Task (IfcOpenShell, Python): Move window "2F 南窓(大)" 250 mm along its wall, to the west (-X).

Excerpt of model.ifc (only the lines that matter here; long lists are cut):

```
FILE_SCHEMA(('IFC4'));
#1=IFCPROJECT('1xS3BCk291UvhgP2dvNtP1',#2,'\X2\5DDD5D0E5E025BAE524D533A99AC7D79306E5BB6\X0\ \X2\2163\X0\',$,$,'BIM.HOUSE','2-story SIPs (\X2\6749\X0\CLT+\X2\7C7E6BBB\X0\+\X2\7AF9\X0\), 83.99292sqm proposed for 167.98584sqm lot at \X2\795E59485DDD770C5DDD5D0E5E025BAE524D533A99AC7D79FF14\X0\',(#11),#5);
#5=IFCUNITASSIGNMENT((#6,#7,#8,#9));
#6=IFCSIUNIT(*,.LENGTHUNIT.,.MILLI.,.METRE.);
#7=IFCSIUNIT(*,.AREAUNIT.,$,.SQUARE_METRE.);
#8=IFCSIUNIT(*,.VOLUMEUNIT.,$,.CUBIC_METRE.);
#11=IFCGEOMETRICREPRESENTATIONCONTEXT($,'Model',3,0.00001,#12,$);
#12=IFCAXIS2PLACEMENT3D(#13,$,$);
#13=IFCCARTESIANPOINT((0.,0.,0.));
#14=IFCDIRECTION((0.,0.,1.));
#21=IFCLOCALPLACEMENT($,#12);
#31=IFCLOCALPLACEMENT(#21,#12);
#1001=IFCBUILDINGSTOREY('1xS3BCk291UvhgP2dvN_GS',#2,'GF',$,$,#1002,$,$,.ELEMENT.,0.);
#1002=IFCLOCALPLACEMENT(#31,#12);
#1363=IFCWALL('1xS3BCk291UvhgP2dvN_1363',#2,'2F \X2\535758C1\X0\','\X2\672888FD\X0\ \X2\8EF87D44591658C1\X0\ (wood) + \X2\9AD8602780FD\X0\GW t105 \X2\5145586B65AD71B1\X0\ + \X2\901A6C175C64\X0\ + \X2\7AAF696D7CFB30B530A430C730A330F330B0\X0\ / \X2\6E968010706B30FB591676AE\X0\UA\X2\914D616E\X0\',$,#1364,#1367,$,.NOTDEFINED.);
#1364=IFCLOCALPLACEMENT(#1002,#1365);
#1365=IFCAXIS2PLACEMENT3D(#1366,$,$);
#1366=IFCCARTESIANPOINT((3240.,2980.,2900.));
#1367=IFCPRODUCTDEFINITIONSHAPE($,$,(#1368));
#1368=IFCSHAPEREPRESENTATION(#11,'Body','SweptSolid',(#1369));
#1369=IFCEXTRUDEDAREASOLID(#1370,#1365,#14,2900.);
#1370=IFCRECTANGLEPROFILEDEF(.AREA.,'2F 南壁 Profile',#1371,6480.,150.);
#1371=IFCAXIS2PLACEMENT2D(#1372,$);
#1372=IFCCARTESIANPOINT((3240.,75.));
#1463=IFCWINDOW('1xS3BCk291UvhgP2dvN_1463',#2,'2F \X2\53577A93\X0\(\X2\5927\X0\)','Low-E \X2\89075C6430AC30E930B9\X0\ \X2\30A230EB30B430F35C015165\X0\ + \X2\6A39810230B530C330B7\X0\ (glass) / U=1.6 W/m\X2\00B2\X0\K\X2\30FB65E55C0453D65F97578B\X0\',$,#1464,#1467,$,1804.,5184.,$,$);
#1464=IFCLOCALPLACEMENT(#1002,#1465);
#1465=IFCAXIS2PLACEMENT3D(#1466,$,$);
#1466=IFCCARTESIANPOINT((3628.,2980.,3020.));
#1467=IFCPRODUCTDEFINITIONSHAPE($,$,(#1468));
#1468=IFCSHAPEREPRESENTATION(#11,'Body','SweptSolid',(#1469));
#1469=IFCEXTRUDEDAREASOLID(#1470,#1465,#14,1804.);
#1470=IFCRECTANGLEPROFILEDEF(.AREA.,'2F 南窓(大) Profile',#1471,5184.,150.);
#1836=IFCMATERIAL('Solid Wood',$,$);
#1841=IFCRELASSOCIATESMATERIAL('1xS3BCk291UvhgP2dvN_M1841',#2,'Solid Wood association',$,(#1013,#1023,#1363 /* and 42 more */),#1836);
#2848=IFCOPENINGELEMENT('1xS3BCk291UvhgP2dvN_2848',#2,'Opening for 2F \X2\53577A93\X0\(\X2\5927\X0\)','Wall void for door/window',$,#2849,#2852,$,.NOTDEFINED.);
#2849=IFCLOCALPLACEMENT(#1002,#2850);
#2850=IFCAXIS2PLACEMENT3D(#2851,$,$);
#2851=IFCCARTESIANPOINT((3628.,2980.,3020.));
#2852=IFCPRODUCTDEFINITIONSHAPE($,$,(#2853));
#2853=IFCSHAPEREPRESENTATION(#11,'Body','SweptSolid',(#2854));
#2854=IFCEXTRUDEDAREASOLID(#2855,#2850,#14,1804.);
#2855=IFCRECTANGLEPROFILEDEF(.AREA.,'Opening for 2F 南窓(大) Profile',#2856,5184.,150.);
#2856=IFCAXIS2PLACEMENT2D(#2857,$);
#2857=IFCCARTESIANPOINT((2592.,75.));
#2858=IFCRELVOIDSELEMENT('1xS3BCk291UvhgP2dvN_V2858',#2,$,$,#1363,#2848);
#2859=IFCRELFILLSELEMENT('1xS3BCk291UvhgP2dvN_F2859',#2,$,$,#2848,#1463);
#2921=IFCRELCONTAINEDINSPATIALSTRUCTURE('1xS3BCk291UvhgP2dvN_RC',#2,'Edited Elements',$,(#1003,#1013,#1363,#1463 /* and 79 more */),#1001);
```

```python
import ifcopenshell
import ifcopenshell.api.geometry
import ifcopenshell.util.placement
import ifcopenshell.util.unit

model = ifcopenshell.open("model.ifc")
unit_scale = ifcopenshell.util.unit.calculate_unit_scale(model)

window = model.by_guid("1xS3BCk291UvhgP2dvN_1463")
opening = window.FillsVoids[0].RelatingOpeningElement
wall = opening.VoidsElements[0].RelatingBuildingElement

wall_matrix = ifcopenshell.util.placement.get_local_placement(wall.ObjectPlacement)
shift = wall_matrix[:3, 0] * -0.25 / unit_scale
before = ifcopenshell.util.placement.get_local_placement(window.ObjectPlacement)[:3, 3].copy()

# The window is not placed relative to its opening, so move both.
for product in (opening, window):
    matrix = ifcopenshell.util.placement.get_local_placement(product.ObjectPlacement)
    matrix[:3, 3] += shift
    ifcopenshell.api.geometry.edit_object_placement(model, product=product, matrix=matrix, is_si=False)

after = ifcopenshell.util.placement.get_local_placement(window.ObjectPlacement)[:3, 3]
print("window moved by", (after - before).round(3) + 0.0)

model.write("model_rev.ifc")
```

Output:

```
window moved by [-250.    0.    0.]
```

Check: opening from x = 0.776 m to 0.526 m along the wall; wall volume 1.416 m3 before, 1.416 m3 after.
